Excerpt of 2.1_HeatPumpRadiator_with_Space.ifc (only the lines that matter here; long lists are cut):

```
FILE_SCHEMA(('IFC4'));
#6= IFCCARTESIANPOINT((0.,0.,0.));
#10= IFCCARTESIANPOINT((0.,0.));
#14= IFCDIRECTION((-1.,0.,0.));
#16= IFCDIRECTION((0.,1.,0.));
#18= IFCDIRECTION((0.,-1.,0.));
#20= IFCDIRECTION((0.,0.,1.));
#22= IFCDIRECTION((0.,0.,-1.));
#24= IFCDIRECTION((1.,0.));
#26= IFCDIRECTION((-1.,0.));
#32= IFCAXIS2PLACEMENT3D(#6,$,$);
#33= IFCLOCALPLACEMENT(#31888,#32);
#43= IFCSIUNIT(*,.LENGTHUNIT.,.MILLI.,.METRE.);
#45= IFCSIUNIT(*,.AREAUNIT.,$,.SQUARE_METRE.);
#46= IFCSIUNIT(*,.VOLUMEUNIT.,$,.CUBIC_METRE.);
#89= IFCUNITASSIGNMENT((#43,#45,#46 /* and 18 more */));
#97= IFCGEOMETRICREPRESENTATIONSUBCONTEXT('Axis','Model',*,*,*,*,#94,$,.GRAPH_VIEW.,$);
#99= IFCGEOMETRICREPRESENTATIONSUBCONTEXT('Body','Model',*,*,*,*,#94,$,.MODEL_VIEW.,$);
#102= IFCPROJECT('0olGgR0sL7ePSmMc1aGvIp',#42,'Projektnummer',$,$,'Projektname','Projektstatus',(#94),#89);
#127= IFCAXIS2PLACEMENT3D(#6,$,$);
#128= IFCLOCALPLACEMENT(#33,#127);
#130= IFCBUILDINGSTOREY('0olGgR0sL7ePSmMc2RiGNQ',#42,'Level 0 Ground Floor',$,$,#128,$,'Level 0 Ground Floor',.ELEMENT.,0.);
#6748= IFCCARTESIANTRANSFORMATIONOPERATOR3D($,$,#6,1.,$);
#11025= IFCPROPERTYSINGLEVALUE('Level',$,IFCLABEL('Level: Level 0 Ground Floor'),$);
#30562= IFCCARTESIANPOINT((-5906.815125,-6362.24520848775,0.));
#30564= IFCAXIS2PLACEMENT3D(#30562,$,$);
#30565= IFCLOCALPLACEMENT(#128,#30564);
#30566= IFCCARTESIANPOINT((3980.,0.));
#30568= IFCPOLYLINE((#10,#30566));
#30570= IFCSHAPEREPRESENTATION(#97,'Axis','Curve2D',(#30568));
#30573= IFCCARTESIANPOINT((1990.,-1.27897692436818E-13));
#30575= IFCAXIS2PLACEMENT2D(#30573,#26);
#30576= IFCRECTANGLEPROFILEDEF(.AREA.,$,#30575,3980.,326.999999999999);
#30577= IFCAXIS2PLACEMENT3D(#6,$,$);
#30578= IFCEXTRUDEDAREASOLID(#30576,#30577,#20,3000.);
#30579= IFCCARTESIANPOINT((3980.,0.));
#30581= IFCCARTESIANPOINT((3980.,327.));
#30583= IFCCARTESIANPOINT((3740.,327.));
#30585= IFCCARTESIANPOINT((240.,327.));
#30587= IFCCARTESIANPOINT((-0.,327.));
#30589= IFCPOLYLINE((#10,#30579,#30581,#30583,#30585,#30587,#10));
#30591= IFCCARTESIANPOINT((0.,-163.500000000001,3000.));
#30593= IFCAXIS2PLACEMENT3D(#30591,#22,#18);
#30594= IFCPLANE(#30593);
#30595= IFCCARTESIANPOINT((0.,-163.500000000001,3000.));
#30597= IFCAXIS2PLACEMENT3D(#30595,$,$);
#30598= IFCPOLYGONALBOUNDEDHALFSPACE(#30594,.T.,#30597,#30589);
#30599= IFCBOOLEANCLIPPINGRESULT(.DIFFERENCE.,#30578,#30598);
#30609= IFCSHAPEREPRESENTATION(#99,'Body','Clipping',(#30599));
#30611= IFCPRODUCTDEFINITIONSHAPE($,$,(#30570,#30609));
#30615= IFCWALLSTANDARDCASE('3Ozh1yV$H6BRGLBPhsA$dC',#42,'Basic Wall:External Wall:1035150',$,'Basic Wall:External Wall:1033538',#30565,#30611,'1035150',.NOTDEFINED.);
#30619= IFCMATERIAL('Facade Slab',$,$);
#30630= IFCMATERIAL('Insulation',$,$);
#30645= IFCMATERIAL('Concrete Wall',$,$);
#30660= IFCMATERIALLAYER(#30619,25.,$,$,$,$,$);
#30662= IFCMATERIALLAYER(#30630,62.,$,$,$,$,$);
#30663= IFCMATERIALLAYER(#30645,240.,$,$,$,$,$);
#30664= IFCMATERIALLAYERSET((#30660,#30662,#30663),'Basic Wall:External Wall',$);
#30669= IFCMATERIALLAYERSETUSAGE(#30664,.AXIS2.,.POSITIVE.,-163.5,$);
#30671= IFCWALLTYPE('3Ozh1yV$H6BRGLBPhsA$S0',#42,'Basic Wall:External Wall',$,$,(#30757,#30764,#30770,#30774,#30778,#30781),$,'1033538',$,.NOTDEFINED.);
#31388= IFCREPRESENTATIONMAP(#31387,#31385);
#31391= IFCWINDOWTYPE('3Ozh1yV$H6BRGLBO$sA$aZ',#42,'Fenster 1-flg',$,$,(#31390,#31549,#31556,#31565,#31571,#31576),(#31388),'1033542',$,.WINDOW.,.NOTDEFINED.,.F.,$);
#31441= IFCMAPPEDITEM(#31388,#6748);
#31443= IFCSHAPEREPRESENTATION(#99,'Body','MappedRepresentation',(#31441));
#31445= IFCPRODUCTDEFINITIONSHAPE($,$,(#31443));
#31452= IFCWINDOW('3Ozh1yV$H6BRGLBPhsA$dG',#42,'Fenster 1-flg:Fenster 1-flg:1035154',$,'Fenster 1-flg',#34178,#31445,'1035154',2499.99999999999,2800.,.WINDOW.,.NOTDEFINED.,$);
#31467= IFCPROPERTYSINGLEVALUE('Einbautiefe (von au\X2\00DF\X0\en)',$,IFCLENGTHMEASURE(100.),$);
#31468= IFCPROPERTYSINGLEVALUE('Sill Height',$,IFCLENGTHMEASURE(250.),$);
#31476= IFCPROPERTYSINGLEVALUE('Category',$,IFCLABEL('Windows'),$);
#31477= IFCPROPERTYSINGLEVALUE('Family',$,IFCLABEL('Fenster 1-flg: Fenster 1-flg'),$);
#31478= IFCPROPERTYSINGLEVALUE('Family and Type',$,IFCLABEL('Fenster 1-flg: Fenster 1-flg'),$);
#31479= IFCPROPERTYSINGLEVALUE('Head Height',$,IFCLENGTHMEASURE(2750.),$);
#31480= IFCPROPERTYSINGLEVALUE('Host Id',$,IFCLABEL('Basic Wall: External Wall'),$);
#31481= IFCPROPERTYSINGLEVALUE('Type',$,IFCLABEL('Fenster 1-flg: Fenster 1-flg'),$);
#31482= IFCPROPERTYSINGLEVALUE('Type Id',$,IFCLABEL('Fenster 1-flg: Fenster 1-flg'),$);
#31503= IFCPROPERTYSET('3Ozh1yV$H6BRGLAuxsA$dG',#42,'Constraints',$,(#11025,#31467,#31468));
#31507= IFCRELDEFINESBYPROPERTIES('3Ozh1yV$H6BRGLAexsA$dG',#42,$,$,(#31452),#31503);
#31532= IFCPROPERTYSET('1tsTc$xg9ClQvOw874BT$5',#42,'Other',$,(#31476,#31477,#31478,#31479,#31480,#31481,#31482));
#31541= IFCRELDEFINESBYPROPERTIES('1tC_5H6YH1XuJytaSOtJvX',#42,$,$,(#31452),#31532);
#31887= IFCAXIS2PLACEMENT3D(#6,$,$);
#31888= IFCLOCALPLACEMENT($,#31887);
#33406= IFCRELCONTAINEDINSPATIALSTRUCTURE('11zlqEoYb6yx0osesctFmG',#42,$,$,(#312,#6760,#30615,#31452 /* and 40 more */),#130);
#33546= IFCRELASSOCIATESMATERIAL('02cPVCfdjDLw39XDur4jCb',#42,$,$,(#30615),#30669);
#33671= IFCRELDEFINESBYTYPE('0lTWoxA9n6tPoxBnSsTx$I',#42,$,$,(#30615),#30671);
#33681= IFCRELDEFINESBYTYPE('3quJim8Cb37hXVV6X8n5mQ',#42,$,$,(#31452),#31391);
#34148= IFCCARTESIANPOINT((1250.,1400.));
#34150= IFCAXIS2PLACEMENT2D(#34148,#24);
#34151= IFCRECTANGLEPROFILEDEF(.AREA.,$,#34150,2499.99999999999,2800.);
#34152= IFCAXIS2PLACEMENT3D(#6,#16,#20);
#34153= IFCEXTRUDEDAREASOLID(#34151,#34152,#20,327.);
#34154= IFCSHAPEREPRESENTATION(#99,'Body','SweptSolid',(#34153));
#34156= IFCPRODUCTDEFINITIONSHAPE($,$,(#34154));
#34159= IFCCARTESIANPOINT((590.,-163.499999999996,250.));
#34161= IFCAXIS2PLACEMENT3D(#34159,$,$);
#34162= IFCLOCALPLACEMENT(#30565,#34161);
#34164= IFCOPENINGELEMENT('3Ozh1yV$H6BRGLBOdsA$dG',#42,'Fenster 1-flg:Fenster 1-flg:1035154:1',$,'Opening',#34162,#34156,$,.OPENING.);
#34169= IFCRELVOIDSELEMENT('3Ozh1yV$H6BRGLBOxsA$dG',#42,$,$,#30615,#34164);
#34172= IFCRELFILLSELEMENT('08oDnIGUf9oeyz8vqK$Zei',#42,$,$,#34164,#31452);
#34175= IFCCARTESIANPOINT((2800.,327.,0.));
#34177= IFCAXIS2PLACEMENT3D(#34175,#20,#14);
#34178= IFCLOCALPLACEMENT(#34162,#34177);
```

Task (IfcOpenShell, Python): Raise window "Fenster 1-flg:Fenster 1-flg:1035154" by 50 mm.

```python
import numpy as np
import ifcopenshell
import ifcopenshell.api.geometry
import ifcopenshell.api.pset
import ifcopenshell.util.element
import ifcopenshell.util.placement
import ifcopenshell.util.unit

model = ifcopenshell.open("2.1_HeatPumpRadiator_with_Space.ifc")
unit_scale = ifcopenshell.util.unit.calculate_unit_scale(model)

window = model.by_id(31452)
opening = window.FillsVoids[0].RelatingOpeningElement
dz = 0.05 / unit_scale

shift = np.array([0.0, 0.0, dz])
# The window is placed relative to its opening, so it follows when the opening moves.
matrix = ifcopenshell.util.placement.get_local_placement(opening.ObjectPlacement)
matrix[:3, 3] += shift
ifcopenshell.api.geometry.edit_object_placement(
    model, product=opening, matrix=matrix, is_si=False, should_transform_children=True
)

# Keep the stored heights in step.
pset = model.by_id(ifcopenshell.util.element.get_pset(window, "Constraints", should_inherit=False)["id"])
ifcopenshell.api.pset.edit_pset(model, pset=pset, properties={
    "Sill Height": model.create_entity("IfcLengthMeasure", ifcopenshell.util.element.get_pset(window, "Constraints", "Sill Height") + dz),
})
pset = model.by_id(ifcopenshell.util.element.get_pset(window, "Other", should_inherit=False)["id"])
ifcopenshell.api.pset.edit_pset(model, pset=pset, properties={
    "Head Height": model.create_entity("IfcLengthMeasure", ifcopenshell.util.element.get_pset(window, "Other", "Head Height") + dz),
})

print(f"moved by {dz * unit_scale:+.3f} m")

model.write("2.1_HeatPumpRadiator_with_Space_v2.ifc")
```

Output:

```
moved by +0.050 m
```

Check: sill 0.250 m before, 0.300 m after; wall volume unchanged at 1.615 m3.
